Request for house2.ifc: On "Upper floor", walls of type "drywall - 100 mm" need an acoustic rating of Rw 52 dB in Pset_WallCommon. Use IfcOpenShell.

First a look at what the model holds.

```python
import ifcopenshell
import ifcopenshell.util.element

model = ifcopenshell.open("house2.ifc")
print(model.schema)
storey = next(s for s in model.by_type("IfcBuildingStorey") if s.Name == "Upper floor")
walls = [e for e in ifcopenshell.util.element.get_decomposition(storey) if e.is_a("IfcWall")]
seen = {}
for e in walls:
    element_type = ifcopenshell.util.element.get_type(e)
    key = (element_type.Name if element_type != e and element_type else None, ifcopenshell.util.element.get_pset(e, "Pset_WallCommon", "AcousticRating"))
    seen[key] = seen.get(key, 0) + 1
for (name, value), count in sorted(seen.items(), key=str):
    print(count, "x", name, "|", value)
```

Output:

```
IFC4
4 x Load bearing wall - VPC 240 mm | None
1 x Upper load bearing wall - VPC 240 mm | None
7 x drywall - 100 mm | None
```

```python
import ifcopenshell
import ifcopenshell.api.pset
import ifcopenshell.util.element

model = ifcopenshell.open("house2.ifc")

storey = next(s for s in model.by_type("IfcBuildingStorey") if s.Name == "Upper floor")
walls = [e for e in ifcopenshell.util.element.get_decomposition(storey) if e.is_a("IfcWall")]

count = 0
for e in walls:
    element_type = ifcopenshell.util.element.get_type(e)
    if element_type in (None, e) or element_type.Name != "drywall - 100 mm":
        continue
    # add_pset returns the element's existing set when there is one.
    pset = ifcopenshell.api.pset.add_pset(model, product=e, name="Pset_WallCommon")
    ifcopenshell.api.pset.edit_pset(model, pset=pset, properties={"AcousticRating": "Rw 52 dB"})
    count += 1

print(count, "walls updated")

model.write("house2_edited.ifc")
```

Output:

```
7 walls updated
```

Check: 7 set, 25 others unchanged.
